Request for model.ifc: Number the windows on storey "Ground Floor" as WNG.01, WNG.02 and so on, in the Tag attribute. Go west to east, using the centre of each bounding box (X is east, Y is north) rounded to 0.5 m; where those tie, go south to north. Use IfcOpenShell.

First a look at what the model holds.

```python
import ifcopenshell
import ifcopenshell.util.element
import ifcopenshell.util.placement

model = ifcopenshell.open("model.ifc")
print(model.schema)
storey = next(s for s in model.by_type("IfcBuildingStorey") if s.Name == "Ground Floor")
windows = [e for e in ifcopenshell.util.element.get_decomposition(storey) if e.is_a("IfcWindow")]
for e in sorted(windows, key=lambda e: e.id()):
    origin = ifcopenshell.util.placement.get_local_placement(e.ObjectPlacement)[:3, 3]
    print(e.id(), e.Tag, e.Name, origin.round(2) + 0.0, sep=" | ")
```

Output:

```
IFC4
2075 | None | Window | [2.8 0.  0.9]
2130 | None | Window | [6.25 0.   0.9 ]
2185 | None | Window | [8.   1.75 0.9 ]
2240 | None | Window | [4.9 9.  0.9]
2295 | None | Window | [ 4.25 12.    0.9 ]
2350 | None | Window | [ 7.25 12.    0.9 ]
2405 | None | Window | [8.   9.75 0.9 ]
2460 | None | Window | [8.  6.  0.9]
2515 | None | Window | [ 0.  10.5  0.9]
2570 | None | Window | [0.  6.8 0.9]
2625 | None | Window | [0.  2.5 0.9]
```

```python
import ifcopenshell
import ifcopenshell.geom
import ifcopenshell.util.element
import ifcopenshell.util.shape

model = ifcopenshell.open("model.ifc")
settings = ifcopenshell.geom.settings()
settings.set("use-world-coords", True)


def centre(element):
    shape = ifcopenshell.geom.create_shape(settings, element)
    return ifcopenshell.util.shape.get_bbox_centroid(shape.geometry)


storey = next(s for s in model.by_type("IfcBuildingStorey") if s.Name == "Ground Floor")
windows = [e for e in ifcopenshell.util.element.get_decomposition(storey) if e.is_a("IfcWindow")]

# Insertion points can sit at a corner or the storey origin, so sort by the geometry (in metres).
centres = {e: centre(e) for e in windows}
windows.sort(key=lambda e: (round(centres[e][0] / 0.5), centres[e][1]))

for i, e in enumerate(windows, start=1):
    number = f"WNG.{i:02d}"
    e.Tag = number
    print(e.id(), number)

model.write("model_rev.ifc")
```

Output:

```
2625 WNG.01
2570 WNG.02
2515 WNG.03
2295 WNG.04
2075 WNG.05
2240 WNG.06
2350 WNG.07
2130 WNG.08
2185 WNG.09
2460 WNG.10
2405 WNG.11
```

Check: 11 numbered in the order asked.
